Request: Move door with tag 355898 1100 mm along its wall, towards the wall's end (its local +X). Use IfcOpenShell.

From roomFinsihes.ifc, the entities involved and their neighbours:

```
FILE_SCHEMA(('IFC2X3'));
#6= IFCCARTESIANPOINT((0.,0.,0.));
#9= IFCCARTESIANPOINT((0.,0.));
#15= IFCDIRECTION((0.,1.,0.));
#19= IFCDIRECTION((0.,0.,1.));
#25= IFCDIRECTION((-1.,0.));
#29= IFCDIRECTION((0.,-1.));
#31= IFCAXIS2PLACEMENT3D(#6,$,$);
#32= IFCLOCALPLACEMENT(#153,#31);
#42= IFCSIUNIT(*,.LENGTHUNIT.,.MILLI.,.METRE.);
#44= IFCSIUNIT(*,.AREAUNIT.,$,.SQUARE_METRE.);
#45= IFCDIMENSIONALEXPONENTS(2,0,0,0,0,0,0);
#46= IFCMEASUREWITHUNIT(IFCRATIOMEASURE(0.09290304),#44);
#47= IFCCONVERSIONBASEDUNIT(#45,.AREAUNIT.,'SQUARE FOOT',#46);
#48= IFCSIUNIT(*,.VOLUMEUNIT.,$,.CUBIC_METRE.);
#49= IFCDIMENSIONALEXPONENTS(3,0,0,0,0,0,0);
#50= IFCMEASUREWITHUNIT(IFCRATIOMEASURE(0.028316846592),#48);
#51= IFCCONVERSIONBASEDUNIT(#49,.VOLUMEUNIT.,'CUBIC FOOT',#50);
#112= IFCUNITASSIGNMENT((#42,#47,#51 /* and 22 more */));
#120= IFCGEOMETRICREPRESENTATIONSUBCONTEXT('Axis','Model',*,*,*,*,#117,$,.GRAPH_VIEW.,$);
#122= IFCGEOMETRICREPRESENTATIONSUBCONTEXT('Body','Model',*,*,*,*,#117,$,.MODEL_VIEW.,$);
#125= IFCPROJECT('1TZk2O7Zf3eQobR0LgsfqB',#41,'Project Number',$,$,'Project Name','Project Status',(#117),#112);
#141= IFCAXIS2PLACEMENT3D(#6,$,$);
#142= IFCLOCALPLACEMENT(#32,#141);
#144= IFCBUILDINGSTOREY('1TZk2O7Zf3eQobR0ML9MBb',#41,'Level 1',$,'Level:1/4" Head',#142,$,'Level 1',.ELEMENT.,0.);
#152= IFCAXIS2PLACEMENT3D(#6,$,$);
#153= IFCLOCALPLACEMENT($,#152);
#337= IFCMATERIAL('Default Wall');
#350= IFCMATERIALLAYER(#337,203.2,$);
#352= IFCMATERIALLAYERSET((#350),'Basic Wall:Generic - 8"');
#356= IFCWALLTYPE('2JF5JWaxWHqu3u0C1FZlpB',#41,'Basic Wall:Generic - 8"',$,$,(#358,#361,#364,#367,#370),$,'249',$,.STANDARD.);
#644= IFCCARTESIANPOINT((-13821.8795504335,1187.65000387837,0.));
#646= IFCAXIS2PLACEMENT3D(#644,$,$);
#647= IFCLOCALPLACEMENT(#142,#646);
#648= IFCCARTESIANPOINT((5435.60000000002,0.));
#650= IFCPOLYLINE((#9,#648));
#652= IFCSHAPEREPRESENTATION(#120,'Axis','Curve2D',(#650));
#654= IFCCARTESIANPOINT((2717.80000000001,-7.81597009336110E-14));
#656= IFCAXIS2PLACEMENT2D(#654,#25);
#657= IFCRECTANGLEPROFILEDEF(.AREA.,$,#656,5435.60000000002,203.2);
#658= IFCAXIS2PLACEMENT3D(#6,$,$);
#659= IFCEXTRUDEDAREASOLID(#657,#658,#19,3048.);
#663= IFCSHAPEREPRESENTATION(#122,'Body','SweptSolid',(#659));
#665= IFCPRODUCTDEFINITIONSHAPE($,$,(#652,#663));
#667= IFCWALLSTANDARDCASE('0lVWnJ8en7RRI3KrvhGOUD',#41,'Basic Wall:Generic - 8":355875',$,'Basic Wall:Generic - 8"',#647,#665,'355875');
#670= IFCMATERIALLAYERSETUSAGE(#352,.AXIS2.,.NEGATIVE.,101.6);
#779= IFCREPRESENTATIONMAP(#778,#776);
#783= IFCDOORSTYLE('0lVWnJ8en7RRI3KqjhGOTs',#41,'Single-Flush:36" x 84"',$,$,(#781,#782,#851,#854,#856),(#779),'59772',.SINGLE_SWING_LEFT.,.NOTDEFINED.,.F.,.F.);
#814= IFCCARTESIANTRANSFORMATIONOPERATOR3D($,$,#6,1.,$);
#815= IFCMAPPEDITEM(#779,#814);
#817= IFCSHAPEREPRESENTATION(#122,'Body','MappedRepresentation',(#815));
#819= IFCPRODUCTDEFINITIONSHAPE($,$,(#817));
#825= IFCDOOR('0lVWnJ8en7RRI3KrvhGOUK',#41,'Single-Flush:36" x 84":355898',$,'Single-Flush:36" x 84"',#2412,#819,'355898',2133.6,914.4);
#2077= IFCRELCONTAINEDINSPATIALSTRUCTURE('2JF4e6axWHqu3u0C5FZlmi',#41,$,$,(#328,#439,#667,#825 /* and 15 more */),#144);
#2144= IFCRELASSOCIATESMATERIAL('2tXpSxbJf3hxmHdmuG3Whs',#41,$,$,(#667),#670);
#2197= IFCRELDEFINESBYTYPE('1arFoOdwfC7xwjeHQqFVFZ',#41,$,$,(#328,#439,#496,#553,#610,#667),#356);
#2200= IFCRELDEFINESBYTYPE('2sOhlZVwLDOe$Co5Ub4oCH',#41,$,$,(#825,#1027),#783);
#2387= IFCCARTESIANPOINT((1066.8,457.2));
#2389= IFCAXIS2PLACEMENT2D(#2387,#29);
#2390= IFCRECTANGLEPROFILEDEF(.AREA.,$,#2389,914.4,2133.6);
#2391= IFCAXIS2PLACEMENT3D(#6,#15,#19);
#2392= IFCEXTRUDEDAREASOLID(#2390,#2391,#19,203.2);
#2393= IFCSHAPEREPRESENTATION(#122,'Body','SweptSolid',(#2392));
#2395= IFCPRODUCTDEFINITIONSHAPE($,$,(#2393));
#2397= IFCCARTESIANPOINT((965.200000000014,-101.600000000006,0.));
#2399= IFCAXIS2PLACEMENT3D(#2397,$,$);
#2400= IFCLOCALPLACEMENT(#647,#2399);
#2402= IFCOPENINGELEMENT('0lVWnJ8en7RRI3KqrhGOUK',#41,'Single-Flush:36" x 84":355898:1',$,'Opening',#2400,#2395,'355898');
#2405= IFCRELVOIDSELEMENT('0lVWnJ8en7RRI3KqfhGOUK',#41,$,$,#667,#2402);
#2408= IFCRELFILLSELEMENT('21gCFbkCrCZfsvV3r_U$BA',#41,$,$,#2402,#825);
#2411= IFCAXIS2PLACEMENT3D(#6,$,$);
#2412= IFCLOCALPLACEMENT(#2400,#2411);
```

```python
import ifcopenshell
import ifcopenshell.api.geometry
import ifcopenshell.util.placement

model = ifcopenshell.open("roomFinsihes.ifc")

door = model.by_guid("0lVWnJ8en7RRI3KrvhGOUK")
opening = door.FillsVoids[0].RelatingOpeningElement
wall = opening.VoidsElements[0].RelatingBuildingElement

wall_matrix = ifcopenshell.util.placement.get_local_placement(wall.ObjectPlacement)
shift = wall_matrix[:3, 0] * 1100.0
before = ifcopenshell.util.placement.get_local_placement(door.ObjectPlacement)[:3, 3].copy()

# The door is placed relative to its opening, so it follows when the opening moves.
matrix = ifcopenshell.util.placement.get_local_placement(opening.ObjectPlacement)
matrix[:3, 3] += shift
ifcopenshell.api.geometry.edit_object_placement(
    model, product=opening, matrix=matrix, is_si=False, should_transform_children=True
)

after = ifcopenshell.util.placement.get_local_placement(door.ObjectPlacement)[:3, 3]
print("door moved by", (after - before).round(3) + 0.0)

model.write("roomFinsihes_v2.ifc")
```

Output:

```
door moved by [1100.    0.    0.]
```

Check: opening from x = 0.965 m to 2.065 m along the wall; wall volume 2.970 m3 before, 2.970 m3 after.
